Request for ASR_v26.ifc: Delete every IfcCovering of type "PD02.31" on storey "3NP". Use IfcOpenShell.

First a look at what the model holds.

```python
import ifcopenshell
import ifcopenshell.util.element

model = ifcopenshell.open("ASR_v26.ifc")
print(model.schema)
storey = next(s for s in model.by_type("IfcBuildingStorey") if s.Name == "3NP")
coverings = [e for e in ifcopenshell.util.element.get_decomposition(storey) if e.is_a("IfcCovering")]
seen = {}
for e in coverings:
    element_type = ifcopenshell.util.element.get_type(e)
    name = element_type.Name if element_type not in (None, e) else None
    seen[name] = seen.get(name, 0) + 1
for name, count in sorted(seen.items(), key=str):
    print(count, "x", name)
```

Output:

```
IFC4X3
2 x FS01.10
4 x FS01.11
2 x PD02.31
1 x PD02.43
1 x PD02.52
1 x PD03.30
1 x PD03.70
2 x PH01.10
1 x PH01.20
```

```python
import ifcopenshell
import ifcopenshell.api.root
import ifcopenshell.util.element

model = ifcopenshell.open("ASR_v26.ifc")

storey = next(s for s in model.by_type("IfcBuildingStorey") if s.Name == "3NP")
coverings = [e for e in ifcopenshell.util.element.get_decomposition(storey) if e.is_a("IfcCovering")]
targets = [e for e in coverings if (t := ifcopenshell.util.element.get_type(e)) not in (None, e) and t.Name == "PD02.31"]

for e in targets:
    ifcopenshell.api.root.remove_product(model, product=e)
print(len(targets), "removed")

model.write("ASR_v26_v2.ifc")
```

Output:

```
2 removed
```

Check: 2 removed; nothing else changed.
